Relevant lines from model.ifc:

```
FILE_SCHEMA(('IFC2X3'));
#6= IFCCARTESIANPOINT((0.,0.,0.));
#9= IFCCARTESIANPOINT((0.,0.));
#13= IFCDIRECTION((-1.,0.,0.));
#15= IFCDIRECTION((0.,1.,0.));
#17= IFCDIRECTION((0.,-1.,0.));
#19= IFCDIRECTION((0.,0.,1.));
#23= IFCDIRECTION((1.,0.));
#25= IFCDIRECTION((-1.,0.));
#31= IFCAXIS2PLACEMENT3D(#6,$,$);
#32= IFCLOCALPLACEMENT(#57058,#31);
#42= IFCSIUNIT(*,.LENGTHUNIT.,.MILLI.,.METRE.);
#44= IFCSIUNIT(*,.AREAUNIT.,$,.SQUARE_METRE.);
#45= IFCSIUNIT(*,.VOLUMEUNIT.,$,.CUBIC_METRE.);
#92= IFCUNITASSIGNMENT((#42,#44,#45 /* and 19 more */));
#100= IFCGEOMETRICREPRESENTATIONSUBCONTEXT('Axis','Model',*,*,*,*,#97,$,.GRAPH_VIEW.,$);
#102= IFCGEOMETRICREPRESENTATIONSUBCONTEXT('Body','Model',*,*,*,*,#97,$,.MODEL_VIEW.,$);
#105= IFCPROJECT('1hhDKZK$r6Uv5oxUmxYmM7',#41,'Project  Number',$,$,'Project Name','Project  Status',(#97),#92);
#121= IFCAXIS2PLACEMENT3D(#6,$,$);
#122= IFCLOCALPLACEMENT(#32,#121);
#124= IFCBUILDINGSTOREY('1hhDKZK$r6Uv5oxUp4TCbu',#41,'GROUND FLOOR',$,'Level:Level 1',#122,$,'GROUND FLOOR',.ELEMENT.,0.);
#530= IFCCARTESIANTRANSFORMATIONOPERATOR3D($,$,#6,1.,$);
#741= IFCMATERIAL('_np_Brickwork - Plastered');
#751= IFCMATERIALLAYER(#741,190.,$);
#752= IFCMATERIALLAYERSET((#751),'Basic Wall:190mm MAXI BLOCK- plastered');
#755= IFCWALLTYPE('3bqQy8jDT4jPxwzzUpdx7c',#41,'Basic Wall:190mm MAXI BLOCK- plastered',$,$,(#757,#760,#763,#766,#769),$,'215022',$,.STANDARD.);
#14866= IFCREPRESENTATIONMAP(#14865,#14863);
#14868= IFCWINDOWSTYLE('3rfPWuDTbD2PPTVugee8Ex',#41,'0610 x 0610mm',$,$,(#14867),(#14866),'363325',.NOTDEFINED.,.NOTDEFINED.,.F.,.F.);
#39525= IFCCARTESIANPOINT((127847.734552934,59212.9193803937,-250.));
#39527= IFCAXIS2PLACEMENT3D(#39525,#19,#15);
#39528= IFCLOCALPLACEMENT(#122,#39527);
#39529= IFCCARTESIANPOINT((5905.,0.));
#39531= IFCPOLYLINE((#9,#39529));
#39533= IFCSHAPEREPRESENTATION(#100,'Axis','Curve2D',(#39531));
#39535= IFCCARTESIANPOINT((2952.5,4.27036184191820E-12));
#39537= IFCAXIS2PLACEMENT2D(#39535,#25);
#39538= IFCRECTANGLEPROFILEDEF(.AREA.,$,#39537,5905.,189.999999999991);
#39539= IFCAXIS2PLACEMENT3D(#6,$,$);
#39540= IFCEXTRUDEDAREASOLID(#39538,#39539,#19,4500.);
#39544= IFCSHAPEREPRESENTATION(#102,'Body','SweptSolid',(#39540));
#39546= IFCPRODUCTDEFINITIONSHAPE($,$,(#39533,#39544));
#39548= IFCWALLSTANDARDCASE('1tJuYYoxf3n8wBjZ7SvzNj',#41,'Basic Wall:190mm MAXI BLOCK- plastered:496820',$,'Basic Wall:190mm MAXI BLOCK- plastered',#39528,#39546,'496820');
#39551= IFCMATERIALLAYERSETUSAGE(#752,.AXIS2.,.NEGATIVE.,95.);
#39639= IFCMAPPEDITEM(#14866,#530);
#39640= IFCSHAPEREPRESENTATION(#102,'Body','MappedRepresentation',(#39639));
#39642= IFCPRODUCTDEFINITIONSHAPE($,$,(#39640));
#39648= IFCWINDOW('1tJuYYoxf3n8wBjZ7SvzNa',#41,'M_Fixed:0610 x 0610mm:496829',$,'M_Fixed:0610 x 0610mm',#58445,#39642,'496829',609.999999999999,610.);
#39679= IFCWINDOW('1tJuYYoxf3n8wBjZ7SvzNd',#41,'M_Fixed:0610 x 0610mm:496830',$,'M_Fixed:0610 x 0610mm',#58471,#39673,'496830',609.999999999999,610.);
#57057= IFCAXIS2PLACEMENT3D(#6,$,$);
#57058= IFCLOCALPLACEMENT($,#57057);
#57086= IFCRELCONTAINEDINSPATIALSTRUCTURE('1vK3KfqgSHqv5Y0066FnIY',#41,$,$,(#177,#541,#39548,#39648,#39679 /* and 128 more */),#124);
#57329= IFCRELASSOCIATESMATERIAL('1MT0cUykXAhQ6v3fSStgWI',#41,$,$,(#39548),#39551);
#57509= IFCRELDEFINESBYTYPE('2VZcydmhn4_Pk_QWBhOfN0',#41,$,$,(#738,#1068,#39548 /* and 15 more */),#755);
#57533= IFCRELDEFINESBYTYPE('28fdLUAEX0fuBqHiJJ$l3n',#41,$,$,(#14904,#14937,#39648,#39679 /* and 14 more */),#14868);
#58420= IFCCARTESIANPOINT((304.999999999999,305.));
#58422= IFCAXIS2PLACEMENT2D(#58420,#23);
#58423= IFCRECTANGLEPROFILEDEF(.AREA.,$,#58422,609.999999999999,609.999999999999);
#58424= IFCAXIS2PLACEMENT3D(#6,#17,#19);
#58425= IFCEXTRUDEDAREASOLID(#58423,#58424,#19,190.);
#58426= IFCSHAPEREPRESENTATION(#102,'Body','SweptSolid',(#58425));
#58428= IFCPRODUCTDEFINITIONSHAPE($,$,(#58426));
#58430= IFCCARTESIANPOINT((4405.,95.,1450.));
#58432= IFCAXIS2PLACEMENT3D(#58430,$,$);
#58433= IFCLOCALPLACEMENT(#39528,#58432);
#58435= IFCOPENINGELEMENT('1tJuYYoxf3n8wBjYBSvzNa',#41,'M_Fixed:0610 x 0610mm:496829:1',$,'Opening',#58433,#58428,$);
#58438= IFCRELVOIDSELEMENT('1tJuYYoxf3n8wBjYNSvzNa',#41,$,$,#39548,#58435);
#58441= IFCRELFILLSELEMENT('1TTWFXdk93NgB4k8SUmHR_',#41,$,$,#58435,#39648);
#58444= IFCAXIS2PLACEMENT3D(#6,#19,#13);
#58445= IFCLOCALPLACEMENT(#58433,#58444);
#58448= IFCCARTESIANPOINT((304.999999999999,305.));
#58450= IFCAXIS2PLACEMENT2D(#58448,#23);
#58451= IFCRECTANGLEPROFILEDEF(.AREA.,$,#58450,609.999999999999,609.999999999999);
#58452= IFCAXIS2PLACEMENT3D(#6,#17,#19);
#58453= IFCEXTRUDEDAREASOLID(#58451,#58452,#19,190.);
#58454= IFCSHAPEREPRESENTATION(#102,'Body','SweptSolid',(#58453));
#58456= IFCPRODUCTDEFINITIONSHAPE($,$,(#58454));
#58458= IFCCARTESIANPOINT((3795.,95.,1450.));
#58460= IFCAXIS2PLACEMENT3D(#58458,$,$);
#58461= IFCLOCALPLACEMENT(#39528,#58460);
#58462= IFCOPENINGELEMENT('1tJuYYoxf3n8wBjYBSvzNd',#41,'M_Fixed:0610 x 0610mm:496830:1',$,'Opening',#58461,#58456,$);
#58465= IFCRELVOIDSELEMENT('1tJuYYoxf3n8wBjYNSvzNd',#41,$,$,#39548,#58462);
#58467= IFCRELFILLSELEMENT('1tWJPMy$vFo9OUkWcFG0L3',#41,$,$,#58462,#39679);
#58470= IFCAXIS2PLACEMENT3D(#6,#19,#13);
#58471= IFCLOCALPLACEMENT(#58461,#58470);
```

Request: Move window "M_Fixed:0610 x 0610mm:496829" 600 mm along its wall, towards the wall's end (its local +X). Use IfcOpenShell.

```python
import ifcopenshell
import ifcopenshell.api.geometry
import ifcopenshell.util.placement
import ifcopenshell.util.unit

model = ifcopenshell.open("model.ifc")
unit_scale = ifcopenshell.util.unit.calculate_unit_scale(model)

window = model.by_id(39648)
opening = window.FillsVoids[0].RelatingOpeningElement
wall = opening.VoidsElements[0].RelatingBuildingElement

wall_matrix = ifcopenshell.util.placement.get_local_placement(wall.ObjectPlacement)
shift = wall_matrix[:3, 0] * 0.6 / unit_scale
before = ifcopenshell.util.placement.get_local_placement(window.ObjectPlacement)[:3, 3].copy()

# The window is placed relative to its opening, so it follows when the opening moves.
matrix = ifcopenshell.util.placement.get_local_placement(opening.ObjectPlacement)
matrix[:3, 3] += shift
ifcopenshell.api.geometry.edit_object_placement(
    model, product=opening, matrix=matrix, is_si=False, should_transform_children=True
)

after = ifcopenshell.util.placement.get_local_placement(window.ObjectPlacement)[:3, 3]
print("window moved by", (after - before).round(3) + 0.0)

model.write("model_updated.ifc")
```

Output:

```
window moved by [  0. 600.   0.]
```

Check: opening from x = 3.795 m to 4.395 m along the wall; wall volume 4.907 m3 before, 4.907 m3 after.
